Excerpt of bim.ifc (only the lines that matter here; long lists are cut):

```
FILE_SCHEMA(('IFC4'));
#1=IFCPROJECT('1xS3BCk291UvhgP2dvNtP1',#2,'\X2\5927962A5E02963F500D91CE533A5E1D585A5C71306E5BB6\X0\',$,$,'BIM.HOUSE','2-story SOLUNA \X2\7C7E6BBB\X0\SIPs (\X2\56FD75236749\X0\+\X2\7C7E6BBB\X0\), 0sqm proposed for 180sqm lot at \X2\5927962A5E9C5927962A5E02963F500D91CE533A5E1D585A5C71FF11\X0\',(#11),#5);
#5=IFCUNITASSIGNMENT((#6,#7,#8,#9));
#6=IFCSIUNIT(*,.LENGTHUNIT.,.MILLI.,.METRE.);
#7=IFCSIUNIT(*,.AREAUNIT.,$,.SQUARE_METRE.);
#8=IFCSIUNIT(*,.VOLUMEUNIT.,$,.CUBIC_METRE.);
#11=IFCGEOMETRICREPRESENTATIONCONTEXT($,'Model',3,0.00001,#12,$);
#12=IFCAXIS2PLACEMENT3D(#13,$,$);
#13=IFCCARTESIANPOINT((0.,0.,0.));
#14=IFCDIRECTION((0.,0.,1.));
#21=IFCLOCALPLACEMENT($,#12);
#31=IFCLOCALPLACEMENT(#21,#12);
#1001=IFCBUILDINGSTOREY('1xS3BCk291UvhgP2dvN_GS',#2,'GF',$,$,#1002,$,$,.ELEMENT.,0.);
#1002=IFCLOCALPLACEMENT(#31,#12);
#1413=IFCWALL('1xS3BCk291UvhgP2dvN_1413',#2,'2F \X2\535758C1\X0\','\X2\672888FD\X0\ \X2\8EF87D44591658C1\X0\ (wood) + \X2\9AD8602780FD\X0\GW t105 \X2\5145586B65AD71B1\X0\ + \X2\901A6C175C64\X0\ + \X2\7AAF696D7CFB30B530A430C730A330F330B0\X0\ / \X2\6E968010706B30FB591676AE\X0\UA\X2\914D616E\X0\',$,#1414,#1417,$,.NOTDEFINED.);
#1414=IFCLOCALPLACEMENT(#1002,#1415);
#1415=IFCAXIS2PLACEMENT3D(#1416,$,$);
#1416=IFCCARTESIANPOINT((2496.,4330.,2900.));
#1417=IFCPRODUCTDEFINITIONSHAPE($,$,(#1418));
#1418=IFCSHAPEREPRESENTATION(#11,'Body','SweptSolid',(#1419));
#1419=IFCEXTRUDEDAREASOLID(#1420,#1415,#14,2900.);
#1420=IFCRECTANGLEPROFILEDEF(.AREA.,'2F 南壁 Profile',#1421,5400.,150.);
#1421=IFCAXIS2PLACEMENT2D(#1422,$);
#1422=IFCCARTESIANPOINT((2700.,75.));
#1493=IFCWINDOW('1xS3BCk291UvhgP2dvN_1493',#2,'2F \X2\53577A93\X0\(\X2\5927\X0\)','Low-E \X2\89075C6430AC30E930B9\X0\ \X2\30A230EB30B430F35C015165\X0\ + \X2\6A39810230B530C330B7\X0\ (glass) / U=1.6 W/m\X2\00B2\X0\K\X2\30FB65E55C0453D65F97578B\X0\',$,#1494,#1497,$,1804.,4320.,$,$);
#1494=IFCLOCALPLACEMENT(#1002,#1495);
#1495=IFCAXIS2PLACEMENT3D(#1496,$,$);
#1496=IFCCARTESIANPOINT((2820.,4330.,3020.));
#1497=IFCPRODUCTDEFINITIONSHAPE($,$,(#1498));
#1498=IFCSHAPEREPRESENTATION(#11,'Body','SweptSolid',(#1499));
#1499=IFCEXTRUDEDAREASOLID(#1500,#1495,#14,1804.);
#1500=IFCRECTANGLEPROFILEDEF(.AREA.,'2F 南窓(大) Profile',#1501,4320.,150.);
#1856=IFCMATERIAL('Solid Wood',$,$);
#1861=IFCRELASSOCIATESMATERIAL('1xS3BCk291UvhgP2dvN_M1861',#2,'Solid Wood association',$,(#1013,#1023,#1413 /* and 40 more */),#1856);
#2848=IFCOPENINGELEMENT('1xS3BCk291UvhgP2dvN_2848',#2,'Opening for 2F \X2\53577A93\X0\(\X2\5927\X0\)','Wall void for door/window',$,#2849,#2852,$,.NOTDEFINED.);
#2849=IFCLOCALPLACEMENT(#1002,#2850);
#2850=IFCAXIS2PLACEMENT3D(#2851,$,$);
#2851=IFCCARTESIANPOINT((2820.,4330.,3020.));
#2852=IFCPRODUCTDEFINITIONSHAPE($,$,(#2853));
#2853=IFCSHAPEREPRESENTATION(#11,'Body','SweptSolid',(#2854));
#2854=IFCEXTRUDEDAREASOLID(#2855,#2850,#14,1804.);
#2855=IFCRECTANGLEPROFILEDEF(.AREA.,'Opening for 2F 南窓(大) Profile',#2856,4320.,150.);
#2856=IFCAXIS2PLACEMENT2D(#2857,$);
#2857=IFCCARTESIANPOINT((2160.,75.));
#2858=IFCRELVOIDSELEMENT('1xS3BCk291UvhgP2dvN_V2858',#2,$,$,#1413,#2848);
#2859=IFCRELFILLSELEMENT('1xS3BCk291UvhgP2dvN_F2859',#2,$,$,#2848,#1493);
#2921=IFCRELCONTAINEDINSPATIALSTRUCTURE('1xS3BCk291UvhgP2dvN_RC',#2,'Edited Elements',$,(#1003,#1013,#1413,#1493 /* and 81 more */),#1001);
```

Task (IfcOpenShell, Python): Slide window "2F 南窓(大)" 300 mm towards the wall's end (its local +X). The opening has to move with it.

```python
import ifcopenshell
import ifcopenshell.api.geometry
import ifcopenshell.util.placement

model = ifcopenshell.open("bim.ifc")

window = model.by_guid("1xS3BCk291UvhgP2dvN_1493")
opening = window.FillsVoids[0].RelatingOpeningElement
wall = opening.VoidsElements[0].RelatingBuildingElement

wall_matrix = ifcopenshell.util.placement.get_local_placement(wall.ObjectPlacement)
shift = wall_matrix[:3, 0] * 300.0
before = ifcopenshell.util.placement.get_local_placement(window.ObjectPlacement)[:3, 3].copy()

# The window is not placed relative to its opening, so move both.
for product in (opening, window):
    matrix = ifcopenshell.util.placement.get_local_placement(product.ObjectPlacement)
    matrix[:3, 3] += shift
    ifcopenshell.api.geometry.edit_object_placement(model, product=product, matrix=matrix, is_si=False)

after = ifcopenshell.util.placement.get_local_placement(window.ObjectPlacement)[:3, 3]
print("window moved by", (after - before).round(3) + 0.0)

model.write("bim_updated.ifc")
```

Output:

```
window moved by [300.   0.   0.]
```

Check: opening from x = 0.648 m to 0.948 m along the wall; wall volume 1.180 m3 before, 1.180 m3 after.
